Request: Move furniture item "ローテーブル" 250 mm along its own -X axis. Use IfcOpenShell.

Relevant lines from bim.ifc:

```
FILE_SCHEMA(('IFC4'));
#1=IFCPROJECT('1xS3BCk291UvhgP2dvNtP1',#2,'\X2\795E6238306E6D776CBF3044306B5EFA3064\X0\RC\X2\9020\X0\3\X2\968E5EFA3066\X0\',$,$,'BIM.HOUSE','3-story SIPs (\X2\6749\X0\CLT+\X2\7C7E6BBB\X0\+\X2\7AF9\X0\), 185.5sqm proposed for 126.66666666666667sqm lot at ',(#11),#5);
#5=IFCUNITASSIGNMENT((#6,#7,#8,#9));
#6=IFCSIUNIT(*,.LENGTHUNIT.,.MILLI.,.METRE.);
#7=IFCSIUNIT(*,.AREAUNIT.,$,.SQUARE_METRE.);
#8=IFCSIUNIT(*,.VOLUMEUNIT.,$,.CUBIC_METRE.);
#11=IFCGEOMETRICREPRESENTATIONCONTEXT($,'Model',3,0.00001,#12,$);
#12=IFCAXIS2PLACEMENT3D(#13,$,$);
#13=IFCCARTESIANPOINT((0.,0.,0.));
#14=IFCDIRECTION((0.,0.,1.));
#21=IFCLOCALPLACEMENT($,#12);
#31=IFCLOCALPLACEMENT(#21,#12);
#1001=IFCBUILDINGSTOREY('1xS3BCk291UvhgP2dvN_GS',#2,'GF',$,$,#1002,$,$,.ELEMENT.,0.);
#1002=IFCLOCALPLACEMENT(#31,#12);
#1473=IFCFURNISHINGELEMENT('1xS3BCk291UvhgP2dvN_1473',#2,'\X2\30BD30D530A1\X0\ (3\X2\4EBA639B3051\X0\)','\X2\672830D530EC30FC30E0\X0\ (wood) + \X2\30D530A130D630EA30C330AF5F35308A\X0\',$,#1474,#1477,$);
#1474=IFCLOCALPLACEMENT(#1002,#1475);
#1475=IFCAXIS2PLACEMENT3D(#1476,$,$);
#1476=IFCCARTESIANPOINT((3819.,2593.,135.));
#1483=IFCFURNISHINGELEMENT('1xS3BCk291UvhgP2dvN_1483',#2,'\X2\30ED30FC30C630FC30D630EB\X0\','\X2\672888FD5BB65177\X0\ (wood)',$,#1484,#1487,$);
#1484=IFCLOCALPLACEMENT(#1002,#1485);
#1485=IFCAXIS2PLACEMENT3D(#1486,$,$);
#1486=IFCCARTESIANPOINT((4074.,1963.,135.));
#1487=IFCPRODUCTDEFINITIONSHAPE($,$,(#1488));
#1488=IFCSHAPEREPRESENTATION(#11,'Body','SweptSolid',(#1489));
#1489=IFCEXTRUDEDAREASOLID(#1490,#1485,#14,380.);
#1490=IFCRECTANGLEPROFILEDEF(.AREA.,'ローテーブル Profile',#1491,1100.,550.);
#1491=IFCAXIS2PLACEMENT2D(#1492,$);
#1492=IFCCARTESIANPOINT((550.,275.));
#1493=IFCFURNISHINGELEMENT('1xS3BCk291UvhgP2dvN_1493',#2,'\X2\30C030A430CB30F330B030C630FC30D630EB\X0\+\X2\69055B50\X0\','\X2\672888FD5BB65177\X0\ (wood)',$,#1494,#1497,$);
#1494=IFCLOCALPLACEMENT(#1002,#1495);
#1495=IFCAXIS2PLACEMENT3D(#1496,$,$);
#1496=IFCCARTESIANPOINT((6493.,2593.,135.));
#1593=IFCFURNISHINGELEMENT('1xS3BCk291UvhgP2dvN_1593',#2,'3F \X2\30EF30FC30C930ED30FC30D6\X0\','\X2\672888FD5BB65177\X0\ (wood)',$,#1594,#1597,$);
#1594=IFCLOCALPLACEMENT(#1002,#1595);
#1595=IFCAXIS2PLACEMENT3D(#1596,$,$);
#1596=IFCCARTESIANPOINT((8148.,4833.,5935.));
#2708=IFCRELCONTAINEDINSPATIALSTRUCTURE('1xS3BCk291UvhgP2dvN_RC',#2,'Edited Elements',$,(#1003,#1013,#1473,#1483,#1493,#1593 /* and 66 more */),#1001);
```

```python
import ifcopenshell
import ifcopenshell.api.geometry
import ifcopenshell.util.placement

model = ifcopenshell.open("bim.ifc")

item = model.by_id(1483)
matrix = ifcopenshell.util.placement.get_local_placement(item.ObjectPlacement)
matrix[:3, 3] -= matrix[:3, 0] * 250.0
ifcopenshell.api.geometry.edit_object_placement(model, product=item, matrix=matrix, is_si=False)

print(ifcopenshell.util.placement.get_local_placement(item.ObjectPlacement).round(3) + 0.0)

model.write("bim-out.ifc")
```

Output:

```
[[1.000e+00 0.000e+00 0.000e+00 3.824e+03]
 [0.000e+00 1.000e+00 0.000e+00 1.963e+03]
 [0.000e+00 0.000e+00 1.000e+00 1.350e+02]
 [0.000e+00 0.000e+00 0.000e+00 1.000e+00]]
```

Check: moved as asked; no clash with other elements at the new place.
